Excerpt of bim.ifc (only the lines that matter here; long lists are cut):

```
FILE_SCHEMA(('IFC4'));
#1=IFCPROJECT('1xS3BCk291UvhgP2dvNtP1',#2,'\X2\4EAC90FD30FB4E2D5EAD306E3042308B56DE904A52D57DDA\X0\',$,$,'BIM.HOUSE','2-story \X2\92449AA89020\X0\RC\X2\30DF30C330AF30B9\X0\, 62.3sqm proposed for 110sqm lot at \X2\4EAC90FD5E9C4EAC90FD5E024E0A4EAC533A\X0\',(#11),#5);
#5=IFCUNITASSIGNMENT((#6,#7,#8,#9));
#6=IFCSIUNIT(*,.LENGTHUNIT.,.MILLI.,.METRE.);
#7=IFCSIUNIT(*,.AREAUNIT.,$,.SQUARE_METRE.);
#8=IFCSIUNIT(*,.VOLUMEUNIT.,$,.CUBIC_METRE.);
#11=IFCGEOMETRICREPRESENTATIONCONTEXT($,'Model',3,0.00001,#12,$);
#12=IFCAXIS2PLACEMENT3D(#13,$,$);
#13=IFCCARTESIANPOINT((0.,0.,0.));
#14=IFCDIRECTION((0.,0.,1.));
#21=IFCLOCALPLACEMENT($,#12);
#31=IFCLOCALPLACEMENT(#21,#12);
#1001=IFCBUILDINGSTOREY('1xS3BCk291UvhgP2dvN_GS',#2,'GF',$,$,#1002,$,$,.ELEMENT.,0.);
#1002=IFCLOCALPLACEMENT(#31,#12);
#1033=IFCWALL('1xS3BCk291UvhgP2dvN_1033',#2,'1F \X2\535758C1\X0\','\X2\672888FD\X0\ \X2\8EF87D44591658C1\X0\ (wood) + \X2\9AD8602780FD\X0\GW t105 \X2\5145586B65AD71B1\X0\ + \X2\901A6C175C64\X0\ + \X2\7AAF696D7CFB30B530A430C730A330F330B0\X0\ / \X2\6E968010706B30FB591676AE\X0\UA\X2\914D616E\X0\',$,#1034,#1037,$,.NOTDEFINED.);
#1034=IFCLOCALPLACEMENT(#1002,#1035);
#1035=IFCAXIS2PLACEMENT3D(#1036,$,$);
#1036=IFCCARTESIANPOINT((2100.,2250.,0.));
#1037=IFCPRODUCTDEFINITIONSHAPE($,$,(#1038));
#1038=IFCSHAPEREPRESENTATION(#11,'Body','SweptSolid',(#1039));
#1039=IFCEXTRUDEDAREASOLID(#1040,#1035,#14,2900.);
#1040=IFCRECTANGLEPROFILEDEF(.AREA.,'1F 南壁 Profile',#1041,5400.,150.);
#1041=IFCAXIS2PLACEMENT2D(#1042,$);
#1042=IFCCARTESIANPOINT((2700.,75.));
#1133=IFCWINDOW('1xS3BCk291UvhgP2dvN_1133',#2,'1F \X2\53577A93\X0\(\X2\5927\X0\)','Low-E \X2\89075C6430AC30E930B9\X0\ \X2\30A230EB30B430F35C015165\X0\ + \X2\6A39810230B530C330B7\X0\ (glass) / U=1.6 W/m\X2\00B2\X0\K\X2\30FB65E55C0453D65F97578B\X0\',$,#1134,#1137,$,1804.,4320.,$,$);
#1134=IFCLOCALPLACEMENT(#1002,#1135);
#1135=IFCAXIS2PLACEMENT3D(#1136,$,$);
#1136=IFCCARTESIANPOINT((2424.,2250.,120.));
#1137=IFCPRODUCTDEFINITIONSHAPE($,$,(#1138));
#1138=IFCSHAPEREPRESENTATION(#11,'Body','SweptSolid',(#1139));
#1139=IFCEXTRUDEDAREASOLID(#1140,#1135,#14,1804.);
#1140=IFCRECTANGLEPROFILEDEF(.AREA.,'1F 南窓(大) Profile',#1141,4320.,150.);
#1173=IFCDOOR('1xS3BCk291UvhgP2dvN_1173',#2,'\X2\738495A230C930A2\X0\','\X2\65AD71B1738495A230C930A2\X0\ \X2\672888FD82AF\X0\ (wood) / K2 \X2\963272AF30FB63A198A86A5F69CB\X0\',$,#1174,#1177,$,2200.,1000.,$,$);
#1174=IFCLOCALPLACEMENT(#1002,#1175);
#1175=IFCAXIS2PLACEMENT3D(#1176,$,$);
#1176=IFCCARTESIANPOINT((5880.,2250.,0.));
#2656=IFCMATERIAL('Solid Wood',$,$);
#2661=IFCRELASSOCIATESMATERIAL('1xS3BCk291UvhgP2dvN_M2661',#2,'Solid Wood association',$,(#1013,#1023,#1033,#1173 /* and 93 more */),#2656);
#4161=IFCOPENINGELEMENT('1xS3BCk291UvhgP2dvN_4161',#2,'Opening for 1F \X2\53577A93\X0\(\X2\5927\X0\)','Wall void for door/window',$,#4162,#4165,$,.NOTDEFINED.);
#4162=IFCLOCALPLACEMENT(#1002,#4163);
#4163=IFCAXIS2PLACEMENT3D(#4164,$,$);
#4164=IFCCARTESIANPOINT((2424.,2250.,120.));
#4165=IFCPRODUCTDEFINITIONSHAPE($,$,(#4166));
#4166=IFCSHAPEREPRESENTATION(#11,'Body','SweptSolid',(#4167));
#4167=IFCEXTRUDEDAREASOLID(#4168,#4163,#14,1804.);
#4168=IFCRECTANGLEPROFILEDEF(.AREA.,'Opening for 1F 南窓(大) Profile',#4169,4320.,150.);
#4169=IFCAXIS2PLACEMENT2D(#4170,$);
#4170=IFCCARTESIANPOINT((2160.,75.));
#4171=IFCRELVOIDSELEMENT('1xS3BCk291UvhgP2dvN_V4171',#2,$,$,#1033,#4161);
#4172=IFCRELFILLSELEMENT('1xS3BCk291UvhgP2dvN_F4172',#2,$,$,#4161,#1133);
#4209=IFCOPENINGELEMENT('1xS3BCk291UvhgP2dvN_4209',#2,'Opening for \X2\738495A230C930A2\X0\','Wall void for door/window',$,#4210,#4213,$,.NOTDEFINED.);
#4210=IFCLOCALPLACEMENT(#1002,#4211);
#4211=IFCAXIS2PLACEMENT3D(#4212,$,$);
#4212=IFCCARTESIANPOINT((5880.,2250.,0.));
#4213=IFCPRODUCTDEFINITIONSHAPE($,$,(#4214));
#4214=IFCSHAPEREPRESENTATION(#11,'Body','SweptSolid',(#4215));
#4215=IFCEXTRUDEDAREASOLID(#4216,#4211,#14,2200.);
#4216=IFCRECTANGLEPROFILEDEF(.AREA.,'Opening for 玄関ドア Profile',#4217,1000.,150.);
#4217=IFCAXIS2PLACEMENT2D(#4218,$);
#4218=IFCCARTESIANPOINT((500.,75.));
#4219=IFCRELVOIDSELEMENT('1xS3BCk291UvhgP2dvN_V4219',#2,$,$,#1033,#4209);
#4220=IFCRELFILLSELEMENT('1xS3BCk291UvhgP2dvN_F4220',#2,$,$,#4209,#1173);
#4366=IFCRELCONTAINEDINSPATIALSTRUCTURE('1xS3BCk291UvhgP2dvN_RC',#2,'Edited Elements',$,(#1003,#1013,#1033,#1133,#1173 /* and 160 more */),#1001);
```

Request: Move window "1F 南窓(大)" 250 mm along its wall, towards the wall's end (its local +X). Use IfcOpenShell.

```python
import ifcopenshell
import ifcopenshell.api.geometry
import ifcopenshell.util.placement

model = ifcopenshell.open("bim.ifc")

window = model.by_guid("1xS3BCk291UvhgP2dvN_1133")
opening = window.FillsVoids[0].RelatingOpeningElement
wall = opening.VoidsElements[0].RelatingBuildingElement

wall_matrix = ifcopenshell.util.placement.get_local_placement(wall.ObjectPlacement)
shift = wall_matrix[:3, 0] * 250.0
before = ifcopenshell.util.placement.get_local_placement(window.ObjectPlacement)[:3, 3].copy()

# The window is not placed relative to its opening, so move both.
for product in (opening, window):
    matrix = ifcopenshell.util.placement.get_local_placement(product.ObjectPlacement)
    matrix[:3, 3] += shift
    ifcopenshell.api.geometry.edit_object_placement(model, product=product, matrix=matrix, is_si=False)

after = ifcopenshell.util.placement.get_local_placement(window.ObjectPlacement)[:3, 3]
print("window moved by", (after - before).round(3) + 0.0)

model.write("bim_updated.ifc")
```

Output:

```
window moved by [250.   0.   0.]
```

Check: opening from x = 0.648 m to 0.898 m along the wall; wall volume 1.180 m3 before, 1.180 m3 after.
